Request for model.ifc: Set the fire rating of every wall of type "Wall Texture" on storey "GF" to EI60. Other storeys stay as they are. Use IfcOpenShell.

First a look at what the model holds.

```python
import ifcopenshell
import ifcopenshell.util.element

model = ifcopenshell.open("model.ifc")
print(model.schema)
storey = next(s for s in model.by_type("IfcBuildingStorey") if s.Name == "GF")
walls = [e for e in ifcopenshell.util.element.get_decomposition(storey) if e.is_a("IfcWall")]
seen = {}
for e in walls:
    element_type = ifcopenshell.util.element.get_type(e)
    key = (element_type.Name if element_type != e and element_type else None, ifcopenshell.util.element.get_pset(e, "Pset_WallCommon", "FireRating"))
    seen[key] = seen.get(key, 0) + 1
for (name, value), count in sorted(seen.items(), key=str):
    print(count, "x", name, "|", value)
```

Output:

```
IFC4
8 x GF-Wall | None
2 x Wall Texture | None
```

```python
import ifcopenshell
import ifcopenshell.api.pset
import ifcopenshell.util.element

model = ifcopenshell.open("model.ifc")

storey = next(s for s in model.by_type("IfcBuildingStorey") if s.Name == "GF")
walls = [e for e in ifcopenshell.util.element.get_decomposition(storey) if e.is_a("IfcWall")]

count = 0
for e in walls:
    element_type = ifcopenshell.util.element.get_type(e)
    if element_type in (None, e) or element_type.Name != "Wall Texture":
        continue
    # add_pset returns the element's existing set when there is one.
    pset = ifcopenshell.api.pset.add_pset(model, product=e, name="Pset_WallCommon")
    ifcopenshell.api.pset.edit_pset(model, pset=pset, properties={"FireRating": "EI60"})
    count += 1

print(count, "walls updated")

model.write("model-out.ifc")
```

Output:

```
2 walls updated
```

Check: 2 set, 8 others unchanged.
